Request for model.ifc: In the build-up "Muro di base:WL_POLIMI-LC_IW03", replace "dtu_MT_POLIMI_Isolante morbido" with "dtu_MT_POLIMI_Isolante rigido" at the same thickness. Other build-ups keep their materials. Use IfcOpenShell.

First a look at what the model holds.

```python
import ifcopenshell
import ifcopenshell.util.element

model = ifcopenshell.open("model.ifc")
print(model.schema)
for layer_set in model.by_type("IfcMaterialLayerSet"):
    if layer_set.LayerSetName == "Muro di base:WL_POLIMI-LC_IW03":
        for layer in layer_set.MaterialLayers:
            print(layer.id(), layer.Material and layer.Material.Name, layer.LayerThickness, sep=" | ")
        print(len(ifcopenshell.util.element.get_elements_by_material(model, layer_set)), "elements and types use it")
print(sorted(m.Name for m in model.by_type("IfcMaterial") if m.Name)[:60])
```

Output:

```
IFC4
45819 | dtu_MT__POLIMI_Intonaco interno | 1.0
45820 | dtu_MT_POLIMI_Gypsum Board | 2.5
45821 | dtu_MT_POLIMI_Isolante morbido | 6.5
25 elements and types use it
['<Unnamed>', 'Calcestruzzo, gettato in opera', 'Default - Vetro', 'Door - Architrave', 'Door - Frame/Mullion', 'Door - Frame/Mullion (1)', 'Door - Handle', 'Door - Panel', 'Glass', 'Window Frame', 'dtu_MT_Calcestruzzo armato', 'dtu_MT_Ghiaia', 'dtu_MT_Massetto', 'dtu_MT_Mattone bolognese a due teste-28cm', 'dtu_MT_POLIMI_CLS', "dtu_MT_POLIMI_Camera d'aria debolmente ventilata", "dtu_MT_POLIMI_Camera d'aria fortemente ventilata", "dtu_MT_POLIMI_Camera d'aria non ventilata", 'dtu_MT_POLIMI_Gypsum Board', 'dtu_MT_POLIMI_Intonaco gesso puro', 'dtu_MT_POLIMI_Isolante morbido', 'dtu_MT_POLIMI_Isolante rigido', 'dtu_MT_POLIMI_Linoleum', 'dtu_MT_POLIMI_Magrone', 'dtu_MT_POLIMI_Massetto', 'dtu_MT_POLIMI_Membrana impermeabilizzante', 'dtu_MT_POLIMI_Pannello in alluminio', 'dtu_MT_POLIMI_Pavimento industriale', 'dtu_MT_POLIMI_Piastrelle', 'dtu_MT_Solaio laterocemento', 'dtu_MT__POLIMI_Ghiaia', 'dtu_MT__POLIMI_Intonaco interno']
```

```python
import ifcopenshell
import ifcopenshell.api.material

model = ifcopenshell.open("model.ifc")

layer_set = next(s for s in model.by_type("IfcMaterialLayerSet") if s.LayerSetName == "Muro di base:WL_POLIMI-LC_IW03")
layer = next(l for l in layer_set.MaterialLayers if l.Material and l.Material.Name == "dtu_MT_POLIMI_Isolante morbido")
material = next(m for m in model.by_type("IfcMaterial") if m.Name == "dtu_MT_POLIMI_Isolante rigido")

# Point this one layer at the other material; renaming the old one would change it everywhere.
ifcopenshell.api.material.edit_layer(model, layer=layer, attributes={"Name": material.Name}, material=material)

print([l.Material.Name if l.Material else None for l in layer_set.MaterialLayers])

model.write("model_rev.ifc")
```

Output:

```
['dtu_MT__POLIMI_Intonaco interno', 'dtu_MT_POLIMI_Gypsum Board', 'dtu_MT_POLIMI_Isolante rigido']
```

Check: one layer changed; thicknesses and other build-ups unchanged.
